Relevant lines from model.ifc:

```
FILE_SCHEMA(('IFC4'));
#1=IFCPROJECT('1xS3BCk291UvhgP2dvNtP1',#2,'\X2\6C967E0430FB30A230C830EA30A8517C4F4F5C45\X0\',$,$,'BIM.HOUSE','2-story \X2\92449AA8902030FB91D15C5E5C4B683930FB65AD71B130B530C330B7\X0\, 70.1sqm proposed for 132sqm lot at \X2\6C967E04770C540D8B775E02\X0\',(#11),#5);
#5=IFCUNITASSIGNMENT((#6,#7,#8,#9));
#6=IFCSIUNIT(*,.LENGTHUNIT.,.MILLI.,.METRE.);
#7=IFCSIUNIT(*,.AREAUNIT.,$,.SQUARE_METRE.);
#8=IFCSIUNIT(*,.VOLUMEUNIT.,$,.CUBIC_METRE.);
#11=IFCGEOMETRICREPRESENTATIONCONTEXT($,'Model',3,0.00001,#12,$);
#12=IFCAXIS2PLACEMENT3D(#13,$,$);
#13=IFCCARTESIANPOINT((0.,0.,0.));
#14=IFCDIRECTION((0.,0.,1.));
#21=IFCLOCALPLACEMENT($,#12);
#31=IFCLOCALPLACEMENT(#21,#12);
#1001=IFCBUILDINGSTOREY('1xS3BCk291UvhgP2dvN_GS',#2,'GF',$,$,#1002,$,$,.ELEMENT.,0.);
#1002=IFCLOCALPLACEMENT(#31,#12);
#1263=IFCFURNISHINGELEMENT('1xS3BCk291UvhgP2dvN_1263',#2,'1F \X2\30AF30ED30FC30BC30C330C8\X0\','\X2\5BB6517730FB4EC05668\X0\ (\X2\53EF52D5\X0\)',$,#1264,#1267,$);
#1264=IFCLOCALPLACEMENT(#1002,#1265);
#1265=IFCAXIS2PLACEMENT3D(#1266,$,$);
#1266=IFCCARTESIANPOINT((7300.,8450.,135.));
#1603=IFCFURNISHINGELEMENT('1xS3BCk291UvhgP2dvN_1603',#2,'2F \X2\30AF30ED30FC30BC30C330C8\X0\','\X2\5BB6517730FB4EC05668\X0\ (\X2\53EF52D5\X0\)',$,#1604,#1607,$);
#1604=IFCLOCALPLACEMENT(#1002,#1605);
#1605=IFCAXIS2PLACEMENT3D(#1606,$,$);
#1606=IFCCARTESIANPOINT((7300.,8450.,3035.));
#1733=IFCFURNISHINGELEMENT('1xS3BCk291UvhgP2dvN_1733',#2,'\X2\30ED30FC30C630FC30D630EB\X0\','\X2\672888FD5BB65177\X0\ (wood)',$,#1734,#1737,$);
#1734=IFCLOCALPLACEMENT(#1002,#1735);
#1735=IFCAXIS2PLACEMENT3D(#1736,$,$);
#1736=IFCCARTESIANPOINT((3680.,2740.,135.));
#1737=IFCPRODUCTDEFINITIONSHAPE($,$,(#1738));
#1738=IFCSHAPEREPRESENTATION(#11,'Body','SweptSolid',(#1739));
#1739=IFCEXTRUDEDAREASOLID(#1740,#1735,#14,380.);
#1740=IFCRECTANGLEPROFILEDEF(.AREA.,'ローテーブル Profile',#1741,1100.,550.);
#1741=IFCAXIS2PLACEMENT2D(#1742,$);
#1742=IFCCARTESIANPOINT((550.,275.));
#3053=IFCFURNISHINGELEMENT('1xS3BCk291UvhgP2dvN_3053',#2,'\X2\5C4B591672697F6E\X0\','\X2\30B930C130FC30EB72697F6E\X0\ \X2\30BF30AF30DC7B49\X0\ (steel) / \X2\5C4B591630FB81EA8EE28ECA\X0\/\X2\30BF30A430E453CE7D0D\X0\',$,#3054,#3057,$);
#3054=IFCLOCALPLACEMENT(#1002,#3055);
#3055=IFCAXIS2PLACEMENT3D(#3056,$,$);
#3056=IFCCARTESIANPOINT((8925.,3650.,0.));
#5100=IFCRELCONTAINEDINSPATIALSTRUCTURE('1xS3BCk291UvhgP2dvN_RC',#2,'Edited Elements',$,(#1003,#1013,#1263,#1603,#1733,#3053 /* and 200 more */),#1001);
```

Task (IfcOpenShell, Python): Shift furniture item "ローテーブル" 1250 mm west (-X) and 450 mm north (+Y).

```python
import ifcopenshell
import ifcopenshell.api.geometry
import ifcopenshell.util.placement

model = ifcopenshell.open("model.ifc")

item = model.by_id(1733)
matrix = ifcopenshell.util.placement.get_local_placement(item.ObjectPlacement)
matrix[0, 3] -= 1250.0
matrix[1, 3] += 450.0
ifcopenshell.api.geometry.edit_object_placement(model, product=item, matrix=matrix, is_si=False)

print(ifcopenshell.util.placement.get_local_placement(item.ObjectPlacement).round(3) + 0.0)

model.write("model_edited.ifc")
```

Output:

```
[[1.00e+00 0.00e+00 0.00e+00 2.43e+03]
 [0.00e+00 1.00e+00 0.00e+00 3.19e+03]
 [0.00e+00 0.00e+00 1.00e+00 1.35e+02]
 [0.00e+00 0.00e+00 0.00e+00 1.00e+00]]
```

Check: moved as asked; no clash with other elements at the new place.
